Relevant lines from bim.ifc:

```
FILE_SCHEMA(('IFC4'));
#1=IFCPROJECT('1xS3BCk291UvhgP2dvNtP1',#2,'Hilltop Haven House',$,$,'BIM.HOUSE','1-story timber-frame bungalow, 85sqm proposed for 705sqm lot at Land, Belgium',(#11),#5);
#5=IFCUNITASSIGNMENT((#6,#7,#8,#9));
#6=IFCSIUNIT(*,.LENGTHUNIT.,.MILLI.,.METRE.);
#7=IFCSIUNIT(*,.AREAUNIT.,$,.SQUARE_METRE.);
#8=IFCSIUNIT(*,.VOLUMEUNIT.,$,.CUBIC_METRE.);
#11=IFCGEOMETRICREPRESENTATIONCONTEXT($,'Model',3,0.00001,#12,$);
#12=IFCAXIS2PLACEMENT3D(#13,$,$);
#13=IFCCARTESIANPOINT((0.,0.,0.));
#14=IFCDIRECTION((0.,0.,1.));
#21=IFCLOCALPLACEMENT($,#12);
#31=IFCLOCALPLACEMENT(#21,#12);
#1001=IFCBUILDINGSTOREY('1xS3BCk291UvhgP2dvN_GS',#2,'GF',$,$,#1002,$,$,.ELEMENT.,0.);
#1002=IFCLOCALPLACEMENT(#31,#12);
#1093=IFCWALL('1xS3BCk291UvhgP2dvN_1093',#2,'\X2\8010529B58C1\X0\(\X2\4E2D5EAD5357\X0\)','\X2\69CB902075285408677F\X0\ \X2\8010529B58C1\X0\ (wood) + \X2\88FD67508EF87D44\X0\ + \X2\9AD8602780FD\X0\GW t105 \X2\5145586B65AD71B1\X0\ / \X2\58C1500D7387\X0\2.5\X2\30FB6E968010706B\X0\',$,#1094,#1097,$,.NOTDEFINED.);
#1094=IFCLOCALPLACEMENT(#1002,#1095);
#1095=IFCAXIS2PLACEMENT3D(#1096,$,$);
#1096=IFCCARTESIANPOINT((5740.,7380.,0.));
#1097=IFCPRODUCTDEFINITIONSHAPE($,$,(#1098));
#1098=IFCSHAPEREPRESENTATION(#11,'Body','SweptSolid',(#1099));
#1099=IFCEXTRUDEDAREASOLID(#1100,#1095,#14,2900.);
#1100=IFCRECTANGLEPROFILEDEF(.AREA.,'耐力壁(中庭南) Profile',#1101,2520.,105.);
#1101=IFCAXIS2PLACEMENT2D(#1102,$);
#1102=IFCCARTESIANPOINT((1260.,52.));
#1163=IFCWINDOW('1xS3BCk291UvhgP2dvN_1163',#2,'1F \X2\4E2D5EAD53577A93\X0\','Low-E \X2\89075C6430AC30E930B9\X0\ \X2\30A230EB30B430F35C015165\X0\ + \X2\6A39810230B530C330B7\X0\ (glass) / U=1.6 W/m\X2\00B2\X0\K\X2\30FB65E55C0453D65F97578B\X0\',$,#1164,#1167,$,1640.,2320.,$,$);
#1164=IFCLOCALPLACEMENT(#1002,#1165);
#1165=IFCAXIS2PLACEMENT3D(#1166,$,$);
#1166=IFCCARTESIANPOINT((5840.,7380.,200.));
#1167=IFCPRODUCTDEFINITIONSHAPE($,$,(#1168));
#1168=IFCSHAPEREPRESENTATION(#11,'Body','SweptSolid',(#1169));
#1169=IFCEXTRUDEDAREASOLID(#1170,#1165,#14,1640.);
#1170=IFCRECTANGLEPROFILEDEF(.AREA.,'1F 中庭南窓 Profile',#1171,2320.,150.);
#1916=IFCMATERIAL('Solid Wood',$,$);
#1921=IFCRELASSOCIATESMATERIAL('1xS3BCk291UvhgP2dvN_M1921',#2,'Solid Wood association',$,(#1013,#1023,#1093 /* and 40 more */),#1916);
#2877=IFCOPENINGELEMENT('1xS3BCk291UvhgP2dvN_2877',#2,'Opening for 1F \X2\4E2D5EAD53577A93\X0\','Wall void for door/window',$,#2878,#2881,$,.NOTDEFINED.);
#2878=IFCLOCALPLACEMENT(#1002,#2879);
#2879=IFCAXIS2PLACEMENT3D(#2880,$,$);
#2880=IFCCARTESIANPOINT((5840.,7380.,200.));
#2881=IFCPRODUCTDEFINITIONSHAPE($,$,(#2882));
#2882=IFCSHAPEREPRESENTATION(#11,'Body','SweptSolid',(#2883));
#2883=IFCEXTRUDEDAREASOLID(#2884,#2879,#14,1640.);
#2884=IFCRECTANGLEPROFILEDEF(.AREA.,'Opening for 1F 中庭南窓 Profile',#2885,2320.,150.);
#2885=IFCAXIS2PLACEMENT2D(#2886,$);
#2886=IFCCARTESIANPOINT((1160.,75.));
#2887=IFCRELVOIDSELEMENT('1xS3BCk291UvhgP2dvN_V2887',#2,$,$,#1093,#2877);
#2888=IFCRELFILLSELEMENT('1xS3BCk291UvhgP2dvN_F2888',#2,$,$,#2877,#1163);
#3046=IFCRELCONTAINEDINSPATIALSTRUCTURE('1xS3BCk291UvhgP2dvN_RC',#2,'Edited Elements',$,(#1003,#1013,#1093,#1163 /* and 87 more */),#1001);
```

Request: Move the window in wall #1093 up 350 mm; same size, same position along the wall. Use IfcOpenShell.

```python
import numpy as np
import ifcopenshell
import ifcopenshell.api.geometry
import ifcopenshell.util.placement
import ifcopenshell.util.unit

model = ifcopenshell.open("bim.ifc")
unit_scale = ifcopenshell.util.unit.calculate_unit_scale(model)

window = model.by_id(1163)
opening = window.FillsVoids[0].RelatingOpeningElement
dz = 0.35 / unit_scale

shift = np.array([0.0, 0.0, dz])
# The window is not placed relative to its opening, so move both.
for product in (opening, window):
    matrix = ifcopenshell.util.placement.get_local_placement(product.ObjectPlacement)
    matrix[:3, 3] += shift
    ifcopenshell.api.geometry.edit_object_placement(model, product=product, matrix=matrix, is_si=False)

print(f"moved by {dz * unit_scale:+.3f} m")

model.write("bim_v2.ifc")
```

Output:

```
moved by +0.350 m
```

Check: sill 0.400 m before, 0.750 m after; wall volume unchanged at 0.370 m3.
